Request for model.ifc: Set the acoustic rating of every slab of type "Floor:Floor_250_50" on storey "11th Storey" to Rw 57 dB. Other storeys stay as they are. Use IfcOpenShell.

First a look at what the model holds.

```python
import ifcopenshell
import ifcopenshell.util.element

model = ifcopenshell.open("model.ifc")
print(model.schema)
storey = next(s for s in model.by_type("IfcBuildingStorey") if s.Name == "11th Storey")
slabs = [e for e in ifcopenshell.util.element.get_decomposition(storey) if e.is_a("IfcSlab")]
seen = {}
for e in slabs:
    element_type = ifcopenshell.util.element.get_type(e)
    key = (element_type.Name if element_type != e and element_type else None, ifcopenshell.util.element.get_pset(e, "Pset_SlabCommon", "AcousticRating"))
    seen[key] = seen.get(key, 0) + 1
for (name, value), count in sorted(seen.items(), key=str):
    print(count, "x", name, "|", value)
```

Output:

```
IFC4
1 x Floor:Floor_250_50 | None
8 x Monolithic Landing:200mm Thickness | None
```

```python
import ifcopenshell
import ifcopenshell.api.pset
import ifcopenshell.util.element

model = ifcopenshell.open("model.ifc")

storey = next(s for s in model.by_type("IfcBuildingStorey") if s.Name == "11th Storey")
slabs = [e for e in ifcopenshell.util.element.get_decomposition(storey) if e.is_a("IfcSlab")]

count = 0
for e in slabs:
    element_type = ifcopenshell.util.element.get_type(e)
    if element_type in (None, e) or element_type.Name != "Floor:Floor_250_50":
        continue
    # add_pset returns the element's existing set when there is one.
    pset = ifcopenshell.api.pset.add_pset(model, product=e, name="Pset_SlabCommon")
    ifcopenshell.api.pset.edit_pset(model, pset=pset, properties={"AcousticRating": "Rw 57 dB"})
    count += 1

print(count, "slabs updated")

model.write("model_rev.ifc")
```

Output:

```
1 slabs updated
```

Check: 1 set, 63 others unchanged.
